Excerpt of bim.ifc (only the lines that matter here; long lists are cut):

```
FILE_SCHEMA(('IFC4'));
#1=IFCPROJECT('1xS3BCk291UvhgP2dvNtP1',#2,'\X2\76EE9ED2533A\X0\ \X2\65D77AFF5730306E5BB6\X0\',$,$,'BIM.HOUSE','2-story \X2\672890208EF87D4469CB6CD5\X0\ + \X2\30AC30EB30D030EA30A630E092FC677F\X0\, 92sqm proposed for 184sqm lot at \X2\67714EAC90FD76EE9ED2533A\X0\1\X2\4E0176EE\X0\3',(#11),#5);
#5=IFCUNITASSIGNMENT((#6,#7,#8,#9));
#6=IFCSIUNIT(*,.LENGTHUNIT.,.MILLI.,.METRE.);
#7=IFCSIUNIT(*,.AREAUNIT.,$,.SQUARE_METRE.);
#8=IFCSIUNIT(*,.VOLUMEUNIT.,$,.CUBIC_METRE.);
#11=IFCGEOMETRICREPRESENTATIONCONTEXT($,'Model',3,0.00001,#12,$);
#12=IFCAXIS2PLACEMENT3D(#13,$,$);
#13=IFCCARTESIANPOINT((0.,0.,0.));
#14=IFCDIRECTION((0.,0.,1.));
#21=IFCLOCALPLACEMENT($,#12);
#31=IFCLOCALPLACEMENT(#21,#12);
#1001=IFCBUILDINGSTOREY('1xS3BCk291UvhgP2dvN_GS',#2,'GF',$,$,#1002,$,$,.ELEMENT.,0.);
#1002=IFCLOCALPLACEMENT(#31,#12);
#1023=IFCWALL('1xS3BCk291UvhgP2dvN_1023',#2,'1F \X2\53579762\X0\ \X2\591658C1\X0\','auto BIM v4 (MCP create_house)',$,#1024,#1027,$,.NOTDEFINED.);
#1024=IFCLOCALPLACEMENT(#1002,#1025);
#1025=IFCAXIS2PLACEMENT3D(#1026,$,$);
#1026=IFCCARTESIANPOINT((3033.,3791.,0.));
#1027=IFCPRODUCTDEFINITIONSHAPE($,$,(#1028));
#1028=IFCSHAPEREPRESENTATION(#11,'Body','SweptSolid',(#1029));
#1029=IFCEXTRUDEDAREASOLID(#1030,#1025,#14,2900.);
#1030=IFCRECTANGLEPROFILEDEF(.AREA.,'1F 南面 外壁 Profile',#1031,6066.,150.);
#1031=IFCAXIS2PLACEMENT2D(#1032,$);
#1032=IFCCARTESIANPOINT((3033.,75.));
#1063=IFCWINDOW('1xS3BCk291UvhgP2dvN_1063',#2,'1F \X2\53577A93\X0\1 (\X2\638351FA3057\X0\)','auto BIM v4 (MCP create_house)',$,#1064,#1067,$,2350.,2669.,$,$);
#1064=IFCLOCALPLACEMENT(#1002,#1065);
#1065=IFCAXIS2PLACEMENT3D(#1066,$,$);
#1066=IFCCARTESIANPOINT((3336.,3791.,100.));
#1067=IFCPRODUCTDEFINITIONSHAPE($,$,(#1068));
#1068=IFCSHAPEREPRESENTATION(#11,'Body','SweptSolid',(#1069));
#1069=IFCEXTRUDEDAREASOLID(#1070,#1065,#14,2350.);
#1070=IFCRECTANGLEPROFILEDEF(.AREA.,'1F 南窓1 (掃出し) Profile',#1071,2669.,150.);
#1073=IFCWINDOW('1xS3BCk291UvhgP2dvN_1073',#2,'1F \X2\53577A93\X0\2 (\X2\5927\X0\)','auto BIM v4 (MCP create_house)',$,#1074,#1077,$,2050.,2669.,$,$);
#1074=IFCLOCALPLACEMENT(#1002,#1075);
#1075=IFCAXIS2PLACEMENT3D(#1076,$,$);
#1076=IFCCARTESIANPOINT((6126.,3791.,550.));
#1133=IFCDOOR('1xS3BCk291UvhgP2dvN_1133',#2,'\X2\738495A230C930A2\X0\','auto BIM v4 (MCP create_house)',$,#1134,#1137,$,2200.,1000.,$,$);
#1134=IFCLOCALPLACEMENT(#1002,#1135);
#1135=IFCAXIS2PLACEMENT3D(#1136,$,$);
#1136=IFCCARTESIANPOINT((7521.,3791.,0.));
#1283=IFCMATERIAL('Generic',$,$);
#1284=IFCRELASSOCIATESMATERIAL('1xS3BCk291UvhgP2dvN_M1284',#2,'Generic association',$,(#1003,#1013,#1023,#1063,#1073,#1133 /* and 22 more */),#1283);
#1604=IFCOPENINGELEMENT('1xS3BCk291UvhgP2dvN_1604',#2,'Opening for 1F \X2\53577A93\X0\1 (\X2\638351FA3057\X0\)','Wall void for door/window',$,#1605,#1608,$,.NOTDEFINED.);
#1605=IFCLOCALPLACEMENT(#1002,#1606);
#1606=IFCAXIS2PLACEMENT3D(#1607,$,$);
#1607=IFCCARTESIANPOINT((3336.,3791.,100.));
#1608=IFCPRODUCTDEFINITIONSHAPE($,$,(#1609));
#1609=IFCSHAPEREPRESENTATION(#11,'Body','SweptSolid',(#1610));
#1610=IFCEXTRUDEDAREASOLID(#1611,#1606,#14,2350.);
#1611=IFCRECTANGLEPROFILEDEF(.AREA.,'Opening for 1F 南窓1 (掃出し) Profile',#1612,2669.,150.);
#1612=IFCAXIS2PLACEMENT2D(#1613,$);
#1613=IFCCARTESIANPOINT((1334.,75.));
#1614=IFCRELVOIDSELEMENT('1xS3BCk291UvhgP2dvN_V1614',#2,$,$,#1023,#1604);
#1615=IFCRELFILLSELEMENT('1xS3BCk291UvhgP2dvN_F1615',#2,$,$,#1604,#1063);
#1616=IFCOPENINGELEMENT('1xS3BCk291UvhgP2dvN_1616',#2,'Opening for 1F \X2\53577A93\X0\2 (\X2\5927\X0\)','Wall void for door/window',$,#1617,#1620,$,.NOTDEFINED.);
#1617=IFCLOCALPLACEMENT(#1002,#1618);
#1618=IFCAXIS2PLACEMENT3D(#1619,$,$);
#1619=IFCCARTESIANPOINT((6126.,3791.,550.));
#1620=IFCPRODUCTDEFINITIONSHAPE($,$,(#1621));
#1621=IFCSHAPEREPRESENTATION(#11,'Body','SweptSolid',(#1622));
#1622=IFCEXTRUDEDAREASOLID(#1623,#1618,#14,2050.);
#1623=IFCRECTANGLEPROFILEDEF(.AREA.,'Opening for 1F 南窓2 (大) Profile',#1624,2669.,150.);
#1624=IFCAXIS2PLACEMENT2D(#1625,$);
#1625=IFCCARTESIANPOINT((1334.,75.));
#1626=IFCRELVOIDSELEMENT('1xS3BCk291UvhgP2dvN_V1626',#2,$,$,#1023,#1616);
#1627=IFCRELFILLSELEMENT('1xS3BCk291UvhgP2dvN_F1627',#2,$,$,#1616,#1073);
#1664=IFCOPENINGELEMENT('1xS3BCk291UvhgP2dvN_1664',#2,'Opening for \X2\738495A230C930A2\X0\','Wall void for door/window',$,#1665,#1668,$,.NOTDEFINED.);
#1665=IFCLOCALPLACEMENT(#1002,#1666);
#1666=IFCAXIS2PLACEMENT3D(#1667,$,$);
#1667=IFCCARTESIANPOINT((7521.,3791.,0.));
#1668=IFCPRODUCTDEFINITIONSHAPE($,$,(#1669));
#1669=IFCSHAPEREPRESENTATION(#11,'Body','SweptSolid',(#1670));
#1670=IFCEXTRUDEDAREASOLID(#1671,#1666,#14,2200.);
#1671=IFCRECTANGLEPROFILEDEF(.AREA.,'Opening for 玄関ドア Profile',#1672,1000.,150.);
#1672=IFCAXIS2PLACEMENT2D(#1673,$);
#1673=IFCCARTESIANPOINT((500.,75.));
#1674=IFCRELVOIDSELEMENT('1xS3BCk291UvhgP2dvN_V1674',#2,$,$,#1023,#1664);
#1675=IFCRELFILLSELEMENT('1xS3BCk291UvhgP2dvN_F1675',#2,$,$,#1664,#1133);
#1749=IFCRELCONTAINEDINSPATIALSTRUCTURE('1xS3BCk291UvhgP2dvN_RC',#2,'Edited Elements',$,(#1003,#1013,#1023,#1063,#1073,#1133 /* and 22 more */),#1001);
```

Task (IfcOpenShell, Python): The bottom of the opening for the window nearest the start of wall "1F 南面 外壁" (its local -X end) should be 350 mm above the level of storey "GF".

```python
import numpy as np
import ifcopenshell
import ifcopenshell.api.geometry
import ifcopenshell.geom
import ifcopenshell.util.element
import ifcopenshell.util.placement
import ifcopenshell.util.shape
import ifcopenshell.util.unit

model = ifcopenshell.open("bim.ifc")
unit_scale = ifcopenshell.util.unit.calculate_unit_scale(model)

window = model.by_id(1063)
opening = window.FillsVoids[0].RelatingOpeningElement
storey = ifcopenshell.util.element.get_container(window, ifc_class="IfcBuildingStorey")
level = ifcopenshell.util.placement.get_local_placement(storey.ObjectPlacement)[2, 3]

# The opening's origin need not be at the sill, so measure its lowest point.
shape = ifcopenshell.geom.create_shape(ifcopenshell.geom.settings(), opening)
bottom = ifcopenshell.util.shape.get_shape_bottom_elevation(shape, shape.geometry) / unit_scale
dz = level + 0.35 / unit_scale - bottom

shift = np.array([0.0, 0.0, dz])
# The window is not placed relative to its opening, so move both.
for product in (opening, window):
    matrix = ifcopenshell.util.placement.get_local_placement(product.ObjectPlacement)
    matrix[:3, 3] += shift
    ifcopenshell.api.geometry.edit_object_placement(model, product=product, matrix=matrix, is_si=False)

print(f"moved by {dz * unit_scale:+.3f} m")

model.write("bim_rev.ifc")
```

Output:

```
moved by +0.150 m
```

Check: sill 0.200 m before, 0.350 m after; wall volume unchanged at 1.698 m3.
